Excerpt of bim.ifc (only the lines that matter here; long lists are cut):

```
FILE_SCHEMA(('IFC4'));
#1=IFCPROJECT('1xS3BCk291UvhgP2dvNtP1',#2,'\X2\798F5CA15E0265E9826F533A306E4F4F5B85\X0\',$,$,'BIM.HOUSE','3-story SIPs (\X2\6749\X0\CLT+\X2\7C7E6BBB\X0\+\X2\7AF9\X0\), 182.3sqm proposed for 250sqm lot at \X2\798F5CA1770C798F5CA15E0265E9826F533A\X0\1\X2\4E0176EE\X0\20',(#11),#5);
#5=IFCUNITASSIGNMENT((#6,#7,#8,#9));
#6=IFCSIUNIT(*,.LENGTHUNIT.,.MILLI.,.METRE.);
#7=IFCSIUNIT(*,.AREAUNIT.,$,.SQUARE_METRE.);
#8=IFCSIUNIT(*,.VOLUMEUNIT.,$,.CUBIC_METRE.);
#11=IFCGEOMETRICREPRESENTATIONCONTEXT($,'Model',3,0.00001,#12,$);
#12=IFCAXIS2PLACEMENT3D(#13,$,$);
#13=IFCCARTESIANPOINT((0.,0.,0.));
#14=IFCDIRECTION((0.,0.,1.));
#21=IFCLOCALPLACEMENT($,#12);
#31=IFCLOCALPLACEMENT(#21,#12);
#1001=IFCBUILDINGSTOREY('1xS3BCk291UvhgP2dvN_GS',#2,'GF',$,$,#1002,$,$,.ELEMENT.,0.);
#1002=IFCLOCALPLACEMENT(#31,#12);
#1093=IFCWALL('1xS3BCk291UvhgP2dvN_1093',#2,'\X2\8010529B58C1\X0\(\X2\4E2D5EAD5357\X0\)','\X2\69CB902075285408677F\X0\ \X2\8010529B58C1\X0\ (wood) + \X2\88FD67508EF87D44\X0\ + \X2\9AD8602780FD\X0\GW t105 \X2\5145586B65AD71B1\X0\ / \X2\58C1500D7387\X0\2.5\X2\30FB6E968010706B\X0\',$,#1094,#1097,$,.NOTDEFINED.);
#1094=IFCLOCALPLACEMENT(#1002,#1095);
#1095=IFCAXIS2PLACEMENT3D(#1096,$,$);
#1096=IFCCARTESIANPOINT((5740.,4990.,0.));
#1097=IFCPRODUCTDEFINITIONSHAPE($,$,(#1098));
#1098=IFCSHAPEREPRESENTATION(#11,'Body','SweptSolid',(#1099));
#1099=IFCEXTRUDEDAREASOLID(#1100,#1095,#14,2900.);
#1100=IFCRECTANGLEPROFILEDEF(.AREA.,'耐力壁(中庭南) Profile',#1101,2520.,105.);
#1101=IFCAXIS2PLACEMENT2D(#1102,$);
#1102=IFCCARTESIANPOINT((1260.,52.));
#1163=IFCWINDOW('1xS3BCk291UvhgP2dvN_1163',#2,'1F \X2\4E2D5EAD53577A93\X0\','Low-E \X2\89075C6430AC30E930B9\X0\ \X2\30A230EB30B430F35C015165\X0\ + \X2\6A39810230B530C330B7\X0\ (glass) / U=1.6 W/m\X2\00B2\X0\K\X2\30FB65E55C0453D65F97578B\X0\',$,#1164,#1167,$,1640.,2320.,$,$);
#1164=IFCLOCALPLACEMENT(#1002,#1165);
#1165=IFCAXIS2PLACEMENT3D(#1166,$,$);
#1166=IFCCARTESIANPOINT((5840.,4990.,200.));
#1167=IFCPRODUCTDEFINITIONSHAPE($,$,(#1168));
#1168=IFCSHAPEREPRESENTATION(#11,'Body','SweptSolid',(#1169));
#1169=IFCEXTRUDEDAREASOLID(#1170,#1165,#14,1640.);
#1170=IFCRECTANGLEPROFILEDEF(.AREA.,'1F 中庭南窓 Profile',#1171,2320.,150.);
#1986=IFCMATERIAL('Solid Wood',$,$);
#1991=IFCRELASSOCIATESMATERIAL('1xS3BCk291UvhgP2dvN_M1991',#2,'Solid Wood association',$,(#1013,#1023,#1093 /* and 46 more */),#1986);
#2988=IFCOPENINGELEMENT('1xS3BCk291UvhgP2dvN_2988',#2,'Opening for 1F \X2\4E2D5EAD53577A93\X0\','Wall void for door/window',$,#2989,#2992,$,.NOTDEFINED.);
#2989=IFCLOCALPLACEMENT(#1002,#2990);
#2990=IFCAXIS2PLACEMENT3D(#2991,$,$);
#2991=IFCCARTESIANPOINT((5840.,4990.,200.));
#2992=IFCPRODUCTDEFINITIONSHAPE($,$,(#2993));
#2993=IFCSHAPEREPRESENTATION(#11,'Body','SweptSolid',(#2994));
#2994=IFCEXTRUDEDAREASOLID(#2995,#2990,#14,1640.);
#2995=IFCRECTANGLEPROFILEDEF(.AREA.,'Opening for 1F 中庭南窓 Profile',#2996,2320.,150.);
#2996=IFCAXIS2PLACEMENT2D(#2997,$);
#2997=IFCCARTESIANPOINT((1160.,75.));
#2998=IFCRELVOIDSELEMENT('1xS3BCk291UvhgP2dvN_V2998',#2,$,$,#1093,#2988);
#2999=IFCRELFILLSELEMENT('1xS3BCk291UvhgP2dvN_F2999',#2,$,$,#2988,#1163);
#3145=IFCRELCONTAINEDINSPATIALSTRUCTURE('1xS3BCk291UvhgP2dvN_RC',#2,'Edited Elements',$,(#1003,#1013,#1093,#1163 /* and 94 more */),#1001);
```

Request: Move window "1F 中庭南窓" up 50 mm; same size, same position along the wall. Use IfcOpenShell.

```python
import numpy as np
import ifcopenshell
import ifcopenshell.api.geometry
import ifcopenshell.util.placement
import ifcopenshell.util.unit

model = ifcopenshell.open("bim.ifc")
unit_scale = ifcopenshell.util.unit.calculate_unit_scale(model)

window = model.by_guid("1xS3BCk291UvhgP2dvN_1163")
opening = window.FillsVoids[0].RelatingOpeningElement
dz = 50.0

shift = np.array([0.0, 0.0, dz])
# The window is not placed relative to its opening, so move both.
for product in (opening, window):
    matrix = ifcopenshell.util.placement.get_local_placement(product.ObjectPlacement)
    matrix[:3, 3] += shift
    ifcopenshell.api.geometry.edit_object_placement(model, product=product, matrix=matrix, is_si=False)

print(f"moved by {dz * unit_scale:+.3f} m")

model.write("bim_rev.ifc")
```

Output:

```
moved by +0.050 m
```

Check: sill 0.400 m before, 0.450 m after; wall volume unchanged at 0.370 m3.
